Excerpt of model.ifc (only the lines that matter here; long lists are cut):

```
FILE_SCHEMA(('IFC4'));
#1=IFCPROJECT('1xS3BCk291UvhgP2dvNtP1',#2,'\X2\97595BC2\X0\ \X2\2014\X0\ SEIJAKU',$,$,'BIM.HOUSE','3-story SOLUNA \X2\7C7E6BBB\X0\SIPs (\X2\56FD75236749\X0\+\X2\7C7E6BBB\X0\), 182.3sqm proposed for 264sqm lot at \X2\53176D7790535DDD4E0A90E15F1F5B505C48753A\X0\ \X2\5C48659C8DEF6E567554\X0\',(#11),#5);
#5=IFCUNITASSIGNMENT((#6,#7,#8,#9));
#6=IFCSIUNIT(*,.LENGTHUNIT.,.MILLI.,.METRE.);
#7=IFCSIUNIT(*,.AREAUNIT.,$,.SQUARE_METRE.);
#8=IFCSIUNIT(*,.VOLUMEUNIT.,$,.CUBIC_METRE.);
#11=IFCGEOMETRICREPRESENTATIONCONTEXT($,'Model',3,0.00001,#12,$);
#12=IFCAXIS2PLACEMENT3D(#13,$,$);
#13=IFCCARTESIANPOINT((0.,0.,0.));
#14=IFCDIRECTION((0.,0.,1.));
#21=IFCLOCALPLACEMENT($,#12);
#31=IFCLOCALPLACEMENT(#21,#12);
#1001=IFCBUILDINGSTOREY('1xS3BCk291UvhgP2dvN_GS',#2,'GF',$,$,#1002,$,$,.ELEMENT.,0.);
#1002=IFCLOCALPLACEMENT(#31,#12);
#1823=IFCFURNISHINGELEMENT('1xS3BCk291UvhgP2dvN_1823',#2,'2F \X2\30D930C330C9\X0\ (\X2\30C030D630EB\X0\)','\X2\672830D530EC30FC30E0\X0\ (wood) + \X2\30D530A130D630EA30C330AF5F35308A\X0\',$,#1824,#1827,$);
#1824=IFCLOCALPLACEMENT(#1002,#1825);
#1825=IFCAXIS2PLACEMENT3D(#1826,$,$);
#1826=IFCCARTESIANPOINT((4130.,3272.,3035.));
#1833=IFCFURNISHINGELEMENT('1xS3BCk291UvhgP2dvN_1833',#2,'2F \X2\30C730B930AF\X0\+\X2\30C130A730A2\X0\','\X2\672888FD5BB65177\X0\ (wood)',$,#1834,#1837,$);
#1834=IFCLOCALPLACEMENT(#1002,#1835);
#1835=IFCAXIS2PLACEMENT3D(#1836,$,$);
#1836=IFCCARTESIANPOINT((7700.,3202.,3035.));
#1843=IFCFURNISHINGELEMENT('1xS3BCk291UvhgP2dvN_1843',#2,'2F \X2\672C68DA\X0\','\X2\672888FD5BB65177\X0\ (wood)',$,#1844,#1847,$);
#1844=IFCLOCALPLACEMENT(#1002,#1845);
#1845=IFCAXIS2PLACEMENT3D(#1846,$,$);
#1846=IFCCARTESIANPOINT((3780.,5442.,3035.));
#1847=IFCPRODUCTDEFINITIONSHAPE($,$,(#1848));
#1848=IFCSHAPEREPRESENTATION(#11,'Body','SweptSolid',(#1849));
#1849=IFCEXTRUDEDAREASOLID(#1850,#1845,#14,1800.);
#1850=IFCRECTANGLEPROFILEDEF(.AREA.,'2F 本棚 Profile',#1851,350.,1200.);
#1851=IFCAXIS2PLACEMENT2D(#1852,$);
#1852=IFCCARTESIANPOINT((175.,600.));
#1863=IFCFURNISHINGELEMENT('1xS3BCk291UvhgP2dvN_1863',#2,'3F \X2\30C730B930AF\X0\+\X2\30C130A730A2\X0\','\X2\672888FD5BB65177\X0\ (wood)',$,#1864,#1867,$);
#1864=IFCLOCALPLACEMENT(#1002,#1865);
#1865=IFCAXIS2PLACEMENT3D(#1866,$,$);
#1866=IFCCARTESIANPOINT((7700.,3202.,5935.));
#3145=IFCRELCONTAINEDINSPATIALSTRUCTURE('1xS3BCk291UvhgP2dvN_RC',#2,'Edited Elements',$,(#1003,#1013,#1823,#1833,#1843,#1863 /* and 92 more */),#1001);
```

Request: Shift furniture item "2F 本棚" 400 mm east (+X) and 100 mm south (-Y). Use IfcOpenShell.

```python
import ifcopenshell
import ifcopenshell.api.geometry
import ifcopenshell.util.placement
import ifcopenshell.util.unit

model = ifcopenshell.open("model.ifc")
unit_scale = ifcopenshell.util.unit.calculate_unit_scale(model)

item = model.by_id(1843)
matrix = ifcopenshell.util.placement.get_local_placement(item.ObjectPlacement)
matrix[0, 3] += 0.4 / unit_scale
matrix[1, 3] -= 0.1 / unit_scale
ifcopenshell.api.geometry.edit_object_placement(model, product=item, matrix=matrix, is_si=False)

print(ifcopenshell.util.placement.get_local_placement(item.ObjectPlacement).round(3) + 0.0)

model.write("model_rev.ifc")
```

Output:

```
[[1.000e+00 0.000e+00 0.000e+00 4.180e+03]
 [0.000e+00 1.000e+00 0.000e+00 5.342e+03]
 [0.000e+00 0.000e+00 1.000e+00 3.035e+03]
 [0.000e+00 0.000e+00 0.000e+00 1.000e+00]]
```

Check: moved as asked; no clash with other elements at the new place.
